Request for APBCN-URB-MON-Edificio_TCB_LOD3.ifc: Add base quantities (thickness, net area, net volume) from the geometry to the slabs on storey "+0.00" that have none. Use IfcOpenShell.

First a look at what the model holds.

```python
import ifcopenshell
import ifcopenshell.util.element
import ifcopenshell.util.unit

model = ifcopenshell.open("APBCN-URB-MON-Edificio_TCB_LOD3.ifc")
print(model.schema)
for unit_type in ("LENGTHUNIT", "AREAUNIT", "VOLUMEUNIT"):
    print(unit_type, ifcopenshell.util.unit.calculate_unit_scale(model, unit_type))
storey = next(s for s in model.by_type("IfcBuildingStorey") if s.Name == "+0.00")
slabs = [e for e in ifcopenshell.util.element.get_decomposition(storey) if e.is_a("IfcSlab")]
for e in sorted(slabs, key=lambda e: e.id()):
    print(e.id(), e.is_a(), e.Name, list(ifcopenshell.util.element.get_psets(e, qtos_only=True)), sep=" | ")
```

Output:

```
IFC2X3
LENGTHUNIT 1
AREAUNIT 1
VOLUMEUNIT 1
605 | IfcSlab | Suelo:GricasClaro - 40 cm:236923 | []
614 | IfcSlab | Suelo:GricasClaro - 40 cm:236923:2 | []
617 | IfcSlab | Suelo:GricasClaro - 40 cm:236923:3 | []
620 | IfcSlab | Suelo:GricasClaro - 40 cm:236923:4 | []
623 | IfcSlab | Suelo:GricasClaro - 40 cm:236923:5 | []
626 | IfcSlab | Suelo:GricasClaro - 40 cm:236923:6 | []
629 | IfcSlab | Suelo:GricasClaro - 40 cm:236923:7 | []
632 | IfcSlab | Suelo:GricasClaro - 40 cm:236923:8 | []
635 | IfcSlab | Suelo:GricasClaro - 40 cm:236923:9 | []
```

```python
import ifcopenshell
import ifcopenshell.api.pset
import ifcopenshell.geom
import ifcopenshell.util.element
import ifcopenshell.util.shape
import ifcopenshell.util.unit

model = ifcopenshell.open("APBCN-URB-MON-Edificio_TCB_LOD3.ifc")
unit_scale = ifcopenshell.util.unit.calculate_unit_scale(model)
area_scale = ifcopenshell.util.unit.calculate_unit_scale(model, "AREAUNIT")
volume_scale = ifcopenshell.util.unit.calculate_unit_scale(model, "VOLUMEUNIT")
settings = ifcopenshell.geom.settings()

storey = next(s for s in model.by_type("IfcBuildingStorey") if s.Name == "+0.00")
slabs = [e for e in ifcopenshell.util.element.get_decomposition(storey) if e.is_a("IfcSlab")]

for e in sorted(slabs, key=lambda e: e.id()):
    if ifcopenshell.util.element.get_psets(e, qtos_only=True, should_inherit=False):
        continue
    # Geometry comes back in metres, in the element's own axes.
    shape = ifcopenshell.geom.create_shape(settings, e)
    values = {
        "Width": ifcopenshell.util.shape.get_z(shape.geometry) / unit_scale,
        "NetArea": ifcopenshell.util.shape.get_footprint_area(shape.geometry) / area_scale,
        "NetVolume": ifcopenshell.util.shape.get_volume(shape.geometry) / volume_scale,
    }
    qto = ifcopenshell.api.pset.add_qto(model, product=e, name="BaseQuantities")
    ifcopenshell.api.pset.edit_qto(model, qto=qto, properties=values)
    print(e.id(), {k: round(v, 3) for k, v in values.items()})

model.write("APBCN-URB-MON-Edificio_TCB_LOD3_v2.ifc")
```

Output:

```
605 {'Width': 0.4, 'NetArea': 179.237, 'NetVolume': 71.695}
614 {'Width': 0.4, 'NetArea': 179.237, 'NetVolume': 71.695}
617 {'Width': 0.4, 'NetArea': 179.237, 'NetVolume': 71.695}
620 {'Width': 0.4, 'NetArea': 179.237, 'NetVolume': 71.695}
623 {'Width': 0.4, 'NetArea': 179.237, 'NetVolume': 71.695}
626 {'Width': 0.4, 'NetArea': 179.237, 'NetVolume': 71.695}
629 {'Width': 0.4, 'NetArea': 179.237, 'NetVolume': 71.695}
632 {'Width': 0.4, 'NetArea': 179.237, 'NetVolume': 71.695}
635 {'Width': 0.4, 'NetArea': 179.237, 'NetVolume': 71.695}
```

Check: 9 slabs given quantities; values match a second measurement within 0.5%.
